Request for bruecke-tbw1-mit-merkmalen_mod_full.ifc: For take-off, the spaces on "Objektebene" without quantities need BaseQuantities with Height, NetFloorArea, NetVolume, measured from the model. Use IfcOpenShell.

First a look at what the model holds.

```python
import ifcopenshell
import ifcopenshell.util.element
import ifcopenshell.util.unit

model = ifcopenshell.open("bruecke-tbw1-mit-merkmalen_mod_full.ifc")
print(model.schema)
for unit_type in ("LENGTHUNIT", "AREAUNIT", "VOLUMEUNIT"):
    print(unit_type, ifcopenshell.util.unit.calculate_unit_scale(model, unit_type))
storey = next(s for s in model.by_type("IfcBuildingStorey") if s.Name == "Objektebene")
spaces = [e for e in ifcopenshell.util.element.get_decomposition(storey) if e.is_a("IfcSpace")]
for e in sorted(spaces, key=lambda e: e.id()):
    print(e.id(), e.is_a(), e.Name, list(ifcopenshell.util.element.get_psets(e, qtos_only=True)), sep=" | ")
```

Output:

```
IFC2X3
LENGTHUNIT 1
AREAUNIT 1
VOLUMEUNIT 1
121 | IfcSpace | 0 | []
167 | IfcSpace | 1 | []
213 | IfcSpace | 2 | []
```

```python
import ifcopenshell
import ifcopenshell.api.pset
import ifcopenshell.geom
import ifcopenshell.util.element
import ifcopenshell.util.shape
import ifcopenshell.util.unit

model = ifcopenshell.open("bruecke-tbw1-mit-merkmalen_mod_full.ifc")
unit_scale = ifcopenshell.util.unit.calculate_unit_scale(model)
area_scale = ifcopenshell.util.unit.calculate_unit_scale(model, "AREAUNIT")
volume_scale = ifcopenshell.util.unit.calculate_unit_scale(model, "VOLUMEUNIT")
settings = ifcopenshell.geom.settings()

storey = next(s for s in model.by_type("IfcBuildingStorey") if s.Name == "Objektebene")
spaces = [e for e in ifcopenshell.util.element.get_decomposition(storey) if e.is_a("IfcSpace")]

for e in sorted(spaces, key=lambda e: e.id()):
    if ifcopenshell.util.element.get_psets(e, qtos_only=True, should_inherit=False):
        continue
    # Geometry comes back in metres, in the element's own axes.
    shape = ifcopenshell.geom.create_shape(settings, e)
    values = {
        "Height": ifcopenshell.util.shape.get_z(shape.geometry) / unit_scale,
        "NetFloorArea": ifcopenshell.util.shape.get_footprint_area(shape.geometry) / area_scale,
        "NetVolume": ifcopenshell.util.shape.get_volume(shape.geometry) / volume_scale,
    }
    qto = ifcopenshell.api.pset.add_qto(model, product=e, name="BaseQuantities")
    ifcopenshell.api.pset.edit_qto(model, qto=qto, properties=values)
    print(e.id(), {k: round(v, 3) for k, v in values.items()})

model.write("bruecke-tbw1-mit-merkmalen_mod_full_updated.ifc")
```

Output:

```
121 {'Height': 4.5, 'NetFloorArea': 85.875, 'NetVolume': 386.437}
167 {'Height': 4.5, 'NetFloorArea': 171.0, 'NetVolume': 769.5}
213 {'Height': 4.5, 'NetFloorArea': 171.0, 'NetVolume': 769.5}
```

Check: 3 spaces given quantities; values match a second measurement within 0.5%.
